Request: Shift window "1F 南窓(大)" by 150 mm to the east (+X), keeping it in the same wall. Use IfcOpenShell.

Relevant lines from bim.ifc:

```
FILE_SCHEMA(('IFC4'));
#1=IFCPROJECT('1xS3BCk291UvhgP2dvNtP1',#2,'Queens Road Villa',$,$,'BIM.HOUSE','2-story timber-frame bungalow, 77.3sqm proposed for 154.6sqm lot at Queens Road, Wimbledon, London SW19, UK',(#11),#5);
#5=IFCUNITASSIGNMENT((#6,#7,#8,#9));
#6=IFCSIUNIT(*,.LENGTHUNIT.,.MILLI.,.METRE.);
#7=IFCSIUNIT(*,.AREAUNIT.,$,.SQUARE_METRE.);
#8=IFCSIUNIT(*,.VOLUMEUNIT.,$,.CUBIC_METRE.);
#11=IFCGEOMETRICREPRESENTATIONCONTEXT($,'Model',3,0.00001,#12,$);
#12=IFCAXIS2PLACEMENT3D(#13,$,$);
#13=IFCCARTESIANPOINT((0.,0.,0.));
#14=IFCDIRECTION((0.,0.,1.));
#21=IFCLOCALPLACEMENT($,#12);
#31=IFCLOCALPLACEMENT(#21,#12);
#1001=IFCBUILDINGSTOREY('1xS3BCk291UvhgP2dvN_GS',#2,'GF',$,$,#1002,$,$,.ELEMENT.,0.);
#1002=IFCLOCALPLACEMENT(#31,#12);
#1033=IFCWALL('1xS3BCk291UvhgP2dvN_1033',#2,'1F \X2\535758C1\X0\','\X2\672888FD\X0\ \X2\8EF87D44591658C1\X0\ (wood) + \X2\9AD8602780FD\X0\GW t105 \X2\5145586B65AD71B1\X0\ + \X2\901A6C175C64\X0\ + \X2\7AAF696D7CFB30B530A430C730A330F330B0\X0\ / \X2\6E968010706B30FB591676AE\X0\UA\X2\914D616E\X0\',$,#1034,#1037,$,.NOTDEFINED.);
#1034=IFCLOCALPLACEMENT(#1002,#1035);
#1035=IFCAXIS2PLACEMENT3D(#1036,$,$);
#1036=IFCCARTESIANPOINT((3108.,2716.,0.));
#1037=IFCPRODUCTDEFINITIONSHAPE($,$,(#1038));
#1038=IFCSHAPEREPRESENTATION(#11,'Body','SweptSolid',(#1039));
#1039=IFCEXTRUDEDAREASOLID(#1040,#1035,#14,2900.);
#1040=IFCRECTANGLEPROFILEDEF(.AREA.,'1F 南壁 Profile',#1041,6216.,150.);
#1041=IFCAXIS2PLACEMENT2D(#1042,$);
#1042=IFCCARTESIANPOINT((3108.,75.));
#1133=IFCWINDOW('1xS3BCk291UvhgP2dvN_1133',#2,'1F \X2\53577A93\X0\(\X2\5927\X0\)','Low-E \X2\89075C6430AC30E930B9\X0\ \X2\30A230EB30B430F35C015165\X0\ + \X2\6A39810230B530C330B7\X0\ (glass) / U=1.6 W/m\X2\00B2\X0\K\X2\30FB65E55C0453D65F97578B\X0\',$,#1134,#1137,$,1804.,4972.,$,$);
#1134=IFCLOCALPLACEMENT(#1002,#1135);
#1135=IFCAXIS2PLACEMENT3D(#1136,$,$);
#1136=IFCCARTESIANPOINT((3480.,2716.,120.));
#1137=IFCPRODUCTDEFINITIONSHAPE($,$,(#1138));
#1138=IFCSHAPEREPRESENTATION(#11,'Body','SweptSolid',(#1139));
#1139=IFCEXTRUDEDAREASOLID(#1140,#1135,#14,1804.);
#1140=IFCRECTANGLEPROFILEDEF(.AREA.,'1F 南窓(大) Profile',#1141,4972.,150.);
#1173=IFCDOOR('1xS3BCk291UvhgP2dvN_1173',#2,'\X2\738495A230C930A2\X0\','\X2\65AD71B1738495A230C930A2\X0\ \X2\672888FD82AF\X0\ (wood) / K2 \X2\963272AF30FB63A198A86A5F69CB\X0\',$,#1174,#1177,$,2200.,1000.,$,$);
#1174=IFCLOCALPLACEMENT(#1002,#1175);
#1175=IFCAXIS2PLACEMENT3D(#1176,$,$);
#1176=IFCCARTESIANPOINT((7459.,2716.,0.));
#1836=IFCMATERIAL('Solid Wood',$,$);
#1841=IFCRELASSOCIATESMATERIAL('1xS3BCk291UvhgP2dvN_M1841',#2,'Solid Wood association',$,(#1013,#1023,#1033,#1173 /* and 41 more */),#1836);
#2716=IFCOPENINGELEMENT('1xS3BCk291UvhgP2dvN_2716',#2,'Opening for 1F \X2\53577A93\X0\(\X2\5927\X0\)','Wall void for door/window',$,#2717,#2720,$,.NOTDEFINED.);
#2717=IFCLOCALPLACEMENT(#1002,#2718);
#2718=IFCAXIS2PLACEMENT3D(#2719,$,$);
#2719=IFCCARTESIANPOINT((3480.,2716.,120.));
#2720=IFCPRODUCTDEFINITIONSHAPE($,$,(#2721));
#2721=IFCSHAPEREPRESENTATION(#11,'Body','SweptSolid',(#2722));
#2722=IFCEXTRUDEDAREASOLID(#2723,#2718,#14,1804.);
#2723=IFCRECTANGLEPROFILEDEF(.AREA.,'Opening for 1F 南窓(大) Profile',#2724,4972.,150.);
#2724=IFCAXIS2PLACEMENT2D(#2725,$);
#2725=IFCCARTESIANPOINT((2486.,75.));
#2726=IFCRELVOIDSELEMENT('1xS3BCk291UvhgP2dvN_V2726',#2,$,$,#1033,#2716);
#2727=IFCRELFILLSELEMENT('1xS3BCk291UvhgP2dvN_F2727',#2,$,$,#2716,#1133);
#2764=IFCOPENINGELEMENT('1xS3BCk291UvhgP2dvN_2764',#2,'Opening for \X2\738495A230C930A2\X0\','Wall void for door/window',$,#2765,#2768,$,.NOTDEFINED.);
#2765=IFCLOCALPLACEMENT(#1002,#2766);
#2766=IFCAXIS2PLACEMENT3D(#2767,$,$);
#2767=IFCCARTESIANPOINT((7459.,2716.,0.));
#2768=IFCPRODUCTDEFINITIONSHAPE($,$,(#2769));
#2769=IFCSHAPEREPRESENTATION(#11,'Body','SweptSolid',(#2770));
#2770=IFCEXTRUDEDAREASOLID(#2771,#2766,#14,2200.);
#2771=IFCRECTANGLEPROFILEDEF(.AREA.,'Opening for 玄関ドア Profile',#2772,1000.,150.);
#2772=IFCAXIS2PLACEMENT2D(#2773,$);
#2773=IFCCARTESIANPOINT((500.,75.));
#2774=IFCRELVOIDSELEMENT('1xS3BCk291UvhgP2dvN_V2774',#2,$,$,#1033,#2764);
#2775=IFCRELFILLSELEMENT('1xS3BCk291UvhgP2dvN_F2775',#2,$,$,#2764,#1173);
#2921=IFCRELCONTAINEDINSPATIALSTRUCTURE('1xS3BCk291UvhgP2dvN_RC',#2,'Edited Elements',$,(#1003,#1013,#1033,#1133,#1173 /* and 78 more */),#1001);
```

```python
import ifcopenshell
import ifcopenshell.api.geometry
import ifcopenshell.util.placement
import ifcopenshell.util.unit

model = ifcopenshell.open("bim.ifc")
unit_scale = ifcopenshell.util.unit.calculate_unit_scale(model)

window = model.by_guid("1xS3BCk291UvhgP2dvN_1133")
opening = window.FillsVoids[0].RelatingOpeningElement
wall = opening.VoidsElements[0].RelatingBuildingElement

wall_matrix = ifcopenshell.util.placement.get_local_placement(wall.ObjectPlacement)
shift = wall_matrix[:3, 0] * 0.15 / unit_scale
before = ifcopenshell.util.placement.get_local_placement(window.ObjectPlacement)[:3, 3].copy()

# The window is not placed relative to its opening, so move both.
for product in (opening, window):
    matrix = ifcopenshell.util.placement.get_local_placement(product.ObjectPlacement)
    matrix[:3, 3] += shift
    ifcopenshell.api.geometry.edit_object_placement(model, product=product, matrix=matrix, is_si=False)

after = ifcopenshell.util.placement.get_local_placement(window.ObjectPlacement)[:3, 3]
print("window moved by", (after - before).round(3) + 0.0)

model.write("bim-out.ifc")
```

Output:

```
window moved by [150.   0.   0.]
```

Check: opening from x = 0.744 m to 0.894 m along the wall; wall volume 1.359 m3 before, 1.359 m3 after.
